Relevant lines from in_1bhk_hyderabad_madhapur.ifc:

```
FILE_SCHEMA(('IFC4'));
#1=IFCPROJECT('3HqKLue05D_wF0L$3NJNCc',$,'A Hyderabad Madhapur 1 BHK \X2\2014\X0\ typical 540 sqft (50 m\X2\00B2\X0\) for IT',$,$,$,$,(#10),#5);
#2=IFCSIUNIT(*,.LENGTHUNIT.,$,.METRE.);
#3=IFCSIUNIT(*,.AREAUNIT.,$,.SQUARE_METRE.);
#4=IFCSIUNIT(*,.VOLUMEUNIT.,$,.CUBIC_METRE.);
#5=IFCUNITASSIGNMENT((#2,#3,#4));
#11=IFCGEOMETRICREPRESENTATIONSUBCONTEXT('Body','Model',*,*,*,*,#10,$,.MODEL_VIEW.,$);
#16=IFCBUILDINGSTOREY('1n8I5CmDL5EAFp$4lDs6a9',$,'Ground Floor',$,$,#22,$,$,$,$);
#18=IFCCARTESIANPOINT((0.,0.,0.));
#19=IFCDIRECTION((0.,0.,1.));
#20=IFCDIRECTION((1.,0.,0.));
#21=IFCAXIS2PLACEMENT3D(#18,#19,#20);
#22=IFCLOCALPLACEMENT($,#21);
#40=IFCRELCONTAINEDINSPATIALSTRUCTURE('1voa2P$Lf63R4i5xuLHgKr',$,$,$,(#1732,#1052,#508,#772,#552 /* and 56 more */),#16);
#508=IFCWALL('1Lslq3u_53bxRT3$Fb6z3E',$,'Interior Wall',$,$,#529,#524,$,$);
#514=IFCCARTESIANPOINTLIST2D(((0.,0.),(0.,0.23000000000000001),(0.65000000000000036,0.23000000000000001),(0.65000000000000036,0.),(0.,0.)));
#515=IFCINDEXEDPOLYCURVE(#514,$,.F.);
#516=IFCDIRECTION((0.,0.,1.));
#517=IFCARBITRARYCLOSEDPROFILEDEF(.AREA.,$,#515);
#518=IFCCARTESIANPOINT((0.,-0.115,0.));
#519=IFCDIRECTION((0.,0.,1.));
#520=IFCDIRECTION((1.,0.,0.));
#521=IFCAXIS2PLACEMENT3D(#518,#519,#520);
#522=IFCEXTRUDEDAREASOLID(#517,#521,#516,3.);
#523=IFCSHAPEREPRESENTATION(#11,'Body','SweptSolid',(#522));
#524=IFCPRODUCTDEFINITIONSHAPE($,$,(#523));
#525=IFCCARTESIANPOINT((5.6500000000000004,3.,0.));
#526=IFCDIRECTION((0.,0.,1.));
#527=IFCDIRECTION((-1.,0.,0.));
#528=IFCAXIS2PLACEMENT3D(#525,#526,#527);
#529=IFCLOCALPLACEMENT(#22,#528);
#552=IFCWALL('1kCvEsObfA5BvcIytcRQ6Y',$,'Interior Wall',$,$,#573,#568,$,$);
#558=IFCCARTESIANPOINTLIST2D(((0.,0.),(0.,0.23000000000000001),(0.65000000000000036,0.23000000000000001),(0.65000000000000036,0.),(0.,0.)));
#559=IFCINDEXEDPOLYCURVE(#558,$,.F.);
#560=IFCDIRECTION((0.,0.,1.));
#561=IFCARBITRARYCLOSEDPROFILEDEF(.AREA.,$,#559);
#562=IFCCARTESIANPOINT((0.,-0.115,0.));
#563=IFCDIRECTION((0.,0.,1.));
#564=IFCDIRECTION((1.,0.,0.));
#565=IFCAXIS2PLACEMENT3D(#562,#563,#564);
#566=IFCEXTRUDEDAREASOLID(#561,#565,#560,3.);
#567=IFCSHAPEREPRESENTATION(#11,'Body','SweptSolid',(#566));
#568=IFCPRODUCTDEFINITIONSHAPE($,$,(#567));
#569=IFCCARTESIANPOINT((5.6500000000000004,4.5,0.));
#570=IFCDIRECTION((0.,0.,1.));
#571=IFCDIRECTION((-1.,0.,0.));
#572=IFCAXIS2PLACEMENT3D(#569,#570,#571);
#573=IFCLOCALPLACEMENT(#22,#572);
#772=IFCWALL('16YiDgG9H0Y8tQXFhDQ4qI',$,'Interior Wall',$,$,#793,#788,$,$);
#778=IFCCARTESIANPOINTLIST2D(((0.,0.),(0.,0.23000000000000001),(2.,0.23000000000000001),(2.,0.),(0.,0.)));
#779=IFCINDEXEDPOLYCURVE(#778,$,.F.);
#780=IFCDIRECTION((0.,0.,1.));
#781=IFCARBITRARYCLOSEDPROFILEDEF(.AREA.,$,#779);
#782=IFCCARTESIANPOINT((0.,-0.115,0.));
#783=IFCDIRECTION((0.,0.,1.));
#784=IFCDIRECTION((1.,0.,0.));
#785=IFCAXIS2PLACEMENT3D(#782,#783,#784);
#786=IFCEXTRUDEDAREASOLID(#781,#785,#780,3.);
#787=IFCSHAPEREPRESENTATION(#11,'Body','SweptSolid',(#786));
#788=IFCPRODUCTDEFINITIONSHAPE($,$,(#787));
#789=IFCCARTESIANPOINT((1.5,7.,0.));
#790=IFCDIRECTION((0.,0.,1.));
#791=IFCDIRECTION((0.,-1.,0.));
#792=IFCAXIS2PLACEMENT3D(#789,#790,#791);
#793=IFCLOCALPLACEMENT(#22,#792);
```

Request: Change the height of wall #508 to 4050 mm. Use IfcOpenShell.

```python
import ifcopenshell
import ifcopenshell.geom
import ifcopenshell.util.representation
import ifcopenshell.util.shape
import ifcopenshell.util.unit

model = ifcopenshell.open("in_1bhk_hyderabad_madhapur.ifc")
unit_scale = ifcopenshell.util.unit.calculate_unit_scale(model)
settings = ifcopenshell.geom.settings()


def volume(element):
    """Net volume in cubic metres, openings subtracted."""
    shape = ifcopenshell.geom.create_shape(settings, element)
    return ifcopenshell.util.shape.get_volume(shape.geometry)


wall = model.by_guid("1Lslq3u_53bxRT3$Fb6z3E")
before = volume(wall)

body = ifcopenshell.util.representation.get_representation(wall, "Model", "Body")
solid = body.Items[0]
old_height = solid.Depth
solid.Depth = 4.05 / unit_scale
after = volume(wall)

print(f"height {old_height:g} -> {solid.Depth:g}, volume {before:.3f} -> {after:.3f} m3")

model.write("in_1bhk_hyderabad_madhapur_updated.ifc")
```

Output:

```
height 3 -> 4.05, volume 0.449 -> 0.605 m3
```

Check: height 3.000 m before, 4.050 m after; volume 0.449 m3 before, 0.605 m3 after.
